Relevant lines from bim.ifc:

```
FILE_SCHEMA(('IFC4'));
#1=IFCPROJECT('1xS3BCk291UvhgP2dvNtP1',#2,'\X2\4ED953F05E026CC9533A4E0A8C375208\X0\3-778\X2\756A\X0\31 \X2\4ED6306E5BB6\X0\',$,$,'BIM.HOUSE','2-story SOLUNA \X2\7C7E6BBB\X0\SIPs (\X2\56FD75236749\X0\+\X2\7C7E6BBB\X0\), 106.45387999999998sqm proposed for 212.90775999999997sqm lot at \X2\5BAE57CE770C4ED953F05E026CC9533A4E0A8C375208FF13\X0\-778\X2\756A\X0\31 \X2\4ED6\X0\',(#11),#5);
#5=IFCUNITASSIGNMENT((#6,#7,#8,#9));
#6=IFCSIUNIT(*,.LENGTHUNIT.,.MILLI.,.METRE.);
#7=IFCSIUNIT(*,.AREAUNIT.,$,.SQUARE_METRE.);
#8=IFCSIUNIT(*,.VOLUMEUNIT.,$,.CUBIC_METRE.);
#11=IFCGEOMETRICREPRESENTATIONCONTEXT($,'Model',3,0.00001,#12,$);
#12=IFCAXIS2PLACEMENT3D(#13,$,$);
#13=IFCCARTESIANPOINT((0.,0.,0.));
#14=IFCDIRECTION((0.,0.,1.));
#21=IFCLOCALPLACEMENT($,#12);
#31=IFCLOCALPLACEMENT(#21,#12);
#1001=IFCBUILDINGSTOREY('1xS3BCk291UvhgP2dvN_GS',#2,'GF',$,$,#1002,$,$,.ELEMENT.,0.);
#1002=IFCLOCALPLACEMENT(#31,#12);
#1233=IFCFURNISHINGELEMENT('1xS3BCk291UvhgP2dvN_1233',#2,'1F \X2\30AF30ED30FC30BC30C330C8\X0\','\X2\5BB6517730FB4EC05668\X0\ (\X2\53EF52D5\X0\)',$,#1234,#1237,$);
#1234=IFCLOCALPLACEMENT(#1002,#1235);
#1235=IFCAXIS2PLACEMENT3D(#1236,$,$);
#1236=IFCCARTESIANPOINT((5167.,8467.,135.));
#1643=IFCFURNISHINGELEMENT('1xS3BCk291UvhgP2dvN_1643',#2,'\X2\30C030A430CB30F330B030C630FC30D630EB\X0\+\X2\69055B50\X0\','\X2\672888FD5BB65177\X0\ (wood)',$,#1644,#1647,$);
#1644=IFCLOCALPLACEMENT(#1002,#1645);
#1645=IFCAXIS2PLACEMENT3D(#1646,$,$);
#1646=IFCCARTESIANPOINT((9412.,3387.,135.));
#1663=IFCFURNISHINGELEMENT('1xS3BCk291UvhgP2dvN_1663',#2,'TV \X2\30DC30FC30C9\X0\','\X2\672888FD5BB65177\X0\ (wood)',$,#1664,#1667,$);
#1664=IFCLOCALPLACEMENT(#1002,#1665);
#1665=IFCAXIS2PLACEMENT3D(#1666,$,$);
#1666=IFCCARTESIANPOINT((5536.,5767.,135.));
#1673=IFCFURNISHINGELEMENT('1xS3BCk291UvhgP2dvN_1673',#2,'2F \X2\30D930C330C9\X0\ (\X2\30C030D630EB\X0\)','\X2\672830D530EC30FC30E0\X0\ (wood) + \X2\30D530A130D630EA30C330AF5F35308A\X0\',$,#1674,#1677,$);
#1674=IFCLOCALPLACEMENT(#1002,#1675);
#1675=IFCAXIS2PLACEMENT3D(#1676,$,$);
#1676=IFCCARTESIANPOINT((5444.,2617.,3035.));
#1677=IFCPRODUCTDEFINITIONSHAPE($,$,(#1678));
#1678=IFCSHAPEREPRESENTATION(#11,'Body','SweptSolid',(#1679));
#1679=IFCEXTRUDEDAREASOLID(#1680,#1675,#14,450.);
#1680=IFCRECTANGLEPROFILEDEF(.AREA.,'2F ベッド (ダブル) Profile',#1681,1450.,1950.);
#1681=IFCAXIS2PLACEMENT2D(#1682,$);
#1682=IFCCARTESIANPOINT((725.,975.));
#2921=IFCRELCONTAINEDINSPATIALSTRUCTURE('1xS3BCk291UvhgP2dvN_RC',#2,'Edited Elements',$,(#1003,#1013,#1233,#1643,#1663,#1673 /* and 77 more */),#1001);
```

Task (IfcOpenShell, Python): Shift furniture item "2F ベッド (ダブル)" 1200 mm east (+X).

```python
import ifcopenshell
import ifcopenshell.api.geometry
import ifcopenshell.util.placement
import ifcopenshell.util.unit

model = ifcopenshell.open("bim.ifc")
unit_scale = ifcopenshell.util.unit.calculate_unit_scale(model)

item = model.by_guid("1xS3BCk291UvhgP2dvN_1673")
matrix = ifcopenshell.util.placement.get_local_placement(item.ObjectPlacement)
matrix[0, 3] += 1.2 / unit_scale
ifcopenshell.api.geometry.edit_object_placement(model, product=item, matrix=matrix, is_si=False)

print(ifcopenshell.util.placement.get_local_placement(item.ObjectPlacement).round(3) + 0.0)

model.write("bim_updated.ifc")
```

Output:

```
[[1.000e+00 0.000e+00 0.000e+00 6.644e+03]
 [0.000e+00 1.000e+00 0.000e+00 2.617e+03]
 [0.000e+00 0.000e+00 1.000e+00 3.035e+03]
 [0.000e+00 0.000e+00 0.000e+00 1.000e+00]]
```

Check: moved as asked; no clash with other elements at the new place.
